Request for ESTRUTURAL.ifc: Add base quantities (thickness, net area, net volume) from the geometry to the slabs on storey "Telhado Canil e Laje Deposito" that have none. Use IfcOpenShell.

First a look at what the model holds.

```python
import ifcopenshell
import ifcopenshell.util.element
import ifcopenshell.util.unit

model = ifcopenshell.open("ESTRUTURAL.ifc")
print(model.schema)
for unit_type in ("LENGTHUNIT", "AREAUNIT", "VOLUMEUNIT"):
    print(unit_type, ifcopenshell.util.unit.calculate_unit_scale(model, unit_type))
storey = next(s for s in model.by_type("IfcBuildingStorey") if s.Name == "Telhado Canil e Laje Deposito")
slabs = [e for e in ifcopenshell.util.element.get_decomposition(storey) if e.is_a("IfcSlab")]
for e in sorted(slabs, key=lambda e: e.id()):
    print(e.id(), e.is_a(), e.Name, list(ifcopenshell.util.element.get_psets(e, qtos_only=True)), sep=" | ")
```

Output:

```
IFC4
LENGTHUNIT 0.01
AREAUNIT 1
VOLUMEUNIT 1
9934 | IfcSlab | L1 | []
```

```python
import ifcopenshell
import ifcopenshell.api.pset
import ifcopenshell.geom
import ifcopenshell.util.element
import ifcopenshell.util.shape
import ifcopenshell.util.unit

model = ifcopenshell.open("ESTRUTURAL.ifc")
unit_scale = ifcopenshell.util.unit.calculate_unit_scale(model)
area_scale = ifcopenshell.util.unit.calculate_unit_scale(model, "AREAUNIT")
volume_scale = ifcopenshell.util.unit.calculate_unit_scale(model, "VOLUMEUNIT")
settings = ifcopenshell.geom.settings()

storey = next(s for s in model.by_type("IfcBuildingStorey") if s.Name == "Telhado Canil e Laje Deposito")
slabs = [e for e in ifcopenshell.util.element.get_decomposition(storey) if e.is_a("IfcSlab")]

for e in sorted(slabs, key=lambda e: e.id()):
    if ifcopenshell.util.element.get_psets(e, qtos_only=True, should_inherit=False):
        continue
    # Geometry comes back in metres, in the element's own axes.
    shape = ifcopenshell.geom.create_shape(settings, e)
    values = {
        "Width": ifcopenshell.util.shape.get_z(shape.geometry) / unit_scale,
        "NetArea": ifcopenshell.util.shape.get_footprint_area(shape.geometry) / area_scale,
        "NetVolume": ifcopenshell.util.shape.get_volume(shape.geometry) / volume_scale,
    }
    qto = ifcopenshell.api.pset.add_qto(model, product=e, name="Qto_SlabBaseQuantities")
    ifcopenshell.api.pset.edit_qto(model, qto=qto, properties=values)
    print(e.id(), {k: round(v, 3) for k, v in values.items()})

model.write("ESTRUTURAL_v2.ifc")
```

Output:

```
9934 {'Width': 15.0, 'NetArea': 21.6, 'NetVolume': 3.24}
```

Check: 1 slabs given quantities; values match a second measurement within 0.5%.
